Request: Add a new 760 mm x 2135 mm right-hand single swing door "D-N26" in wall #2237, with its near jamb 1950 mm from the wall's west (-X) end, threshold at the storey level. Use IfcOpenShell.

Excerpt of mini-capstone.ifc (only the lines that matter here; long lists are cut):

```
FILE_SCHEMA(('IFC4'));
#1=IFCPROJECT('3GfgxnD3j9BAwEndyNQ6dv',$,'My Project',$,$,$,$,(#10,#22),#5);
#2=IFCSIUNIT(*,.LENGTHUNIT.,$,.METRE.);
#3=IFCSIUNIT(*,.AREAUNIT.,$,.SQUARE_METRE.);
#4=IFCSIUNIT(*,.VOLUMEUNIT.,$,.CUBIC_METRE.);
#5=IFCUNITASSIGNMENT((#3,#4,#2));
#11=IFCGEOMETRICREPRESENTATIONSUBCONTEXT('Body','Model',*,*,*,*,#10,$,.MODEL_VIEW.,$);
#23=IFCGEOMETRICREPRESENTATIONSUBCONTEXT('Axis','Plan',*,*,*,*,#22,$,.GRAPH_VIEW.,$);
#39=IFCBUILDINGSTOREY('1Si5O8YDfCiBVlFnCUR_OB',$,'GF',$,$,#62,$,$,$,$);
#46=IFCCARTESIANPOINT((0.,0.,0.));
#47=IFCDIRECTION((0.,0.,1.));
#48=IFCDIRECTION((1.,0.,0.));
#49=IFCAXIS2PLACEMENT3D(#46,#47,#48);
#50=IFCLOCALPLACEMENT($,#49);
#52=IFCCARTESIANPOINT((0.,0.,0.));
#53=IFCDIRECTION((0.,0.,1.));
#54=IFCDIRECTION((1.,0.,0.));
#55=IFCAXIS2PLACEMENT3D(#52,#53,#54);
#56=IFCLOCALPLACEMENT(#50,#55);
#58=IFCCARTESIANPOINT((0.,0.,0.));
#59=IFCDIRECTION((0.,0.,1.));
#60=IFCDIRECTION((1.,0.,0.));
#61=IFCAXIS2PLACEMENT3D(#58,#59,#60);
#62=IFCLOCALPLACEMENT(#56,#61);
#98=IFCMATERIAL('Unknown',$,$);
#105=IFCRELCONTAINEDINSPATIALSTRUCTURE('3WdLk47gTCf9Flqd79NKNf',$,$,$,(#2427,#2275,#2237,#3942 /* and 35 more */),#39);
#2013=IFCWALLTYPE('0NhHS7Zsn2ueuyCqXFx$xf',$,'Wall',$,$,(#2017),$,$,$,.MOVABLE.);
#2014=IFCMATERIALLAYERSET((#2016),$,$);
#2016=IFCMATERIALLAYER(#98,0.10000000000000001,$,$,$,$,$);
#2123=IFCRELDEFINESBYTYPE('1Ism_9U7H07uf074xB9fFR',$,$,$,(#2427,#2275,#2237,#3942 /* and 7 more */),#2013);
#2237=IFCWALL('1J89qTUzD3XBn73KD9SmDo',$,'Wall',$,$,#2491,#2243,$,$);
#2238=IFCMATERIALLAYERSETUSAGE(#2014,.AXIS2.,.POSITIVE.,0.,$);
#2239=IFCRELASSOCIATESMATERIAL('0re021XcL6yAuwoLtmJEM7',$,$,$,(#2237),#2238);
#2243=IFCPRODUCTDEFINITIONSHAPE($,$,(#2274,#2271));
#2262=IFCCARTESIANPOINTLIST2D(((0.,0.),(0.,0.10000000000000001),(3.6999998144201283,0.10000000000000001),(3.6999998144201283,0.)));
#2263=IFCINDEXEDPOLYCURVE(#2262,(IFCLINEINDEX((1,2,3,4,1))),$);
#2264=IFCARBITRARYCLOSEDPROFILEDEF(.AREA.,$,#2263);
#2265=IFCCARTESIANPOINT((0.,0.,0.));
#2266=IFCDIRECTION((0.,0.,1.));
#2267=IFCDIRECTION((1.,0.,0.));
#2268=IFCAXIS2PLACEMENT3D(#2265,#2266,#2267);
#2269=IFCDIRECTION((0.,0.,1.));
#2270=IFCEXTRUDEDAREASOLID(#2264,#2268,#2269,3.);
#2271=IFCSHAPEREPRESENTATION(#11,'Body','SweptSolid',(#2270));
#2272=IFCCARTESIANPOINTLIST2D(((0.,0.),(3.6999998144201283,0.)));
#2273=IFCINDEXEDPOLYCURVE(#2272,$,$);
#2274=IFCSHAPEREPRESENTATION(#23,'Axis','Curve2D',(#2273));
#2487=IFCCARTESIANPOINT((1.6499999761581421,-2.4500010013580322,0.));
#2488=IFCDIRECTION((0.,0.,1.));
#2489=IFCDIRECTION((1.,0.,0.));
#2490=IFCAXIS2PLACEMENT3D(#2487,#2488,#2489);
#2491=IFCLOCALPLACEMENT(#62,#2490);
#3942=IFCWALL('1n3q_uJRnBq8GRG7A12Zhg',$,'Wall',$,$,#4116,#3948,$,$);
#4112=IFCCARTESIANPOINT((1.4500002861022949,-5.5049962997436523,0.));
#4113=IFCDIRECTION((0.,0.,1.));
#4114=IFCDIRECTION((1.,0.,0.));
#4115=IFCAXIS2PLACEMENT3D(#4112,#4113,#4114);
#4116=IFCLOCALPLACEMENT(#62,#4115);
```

```python
import numpy as np
import ifcopenshell
import ifcopenshell.api.feature
import ifcopenshell.api.geometry
import ifcopenshell.api.root
import ifcopenshell.api.spatial
import ifcopenshell.geom
import ifcopenshell.util.element
import ifcopenshell.util.placement
import ifcopenshell.util.representation
import ifcopenshell.util.shape
import ifcopenshell.util.unit

model = ifcopenshell.open("mini-capstone.ifc")
unit_scale = ifcopenshell.util.unit.calculate_unit_scale(model)
settings = ifcopenshell.geom.settings()


def volume(element):
    """Net volume in cubic metres, openings subtracted."""
    shape = ifcopenshell.geom.create_shape(settings, element)
    return ifcopenshell.util.shape.get_volume(shape.geometry)


wall = model.by_guid("1J89qTUzD3XBn73KD9SmDo")
storey = ifcopenshell.util.element.get_container(wall, ifc_class="IfcBuildingStorey")
context = ifcopenshell.util.representation.get_context(model, "Model", "Body", "MODEL_VIEW")
before = volume(wall)

width, height, from_end, sill = 0.76, 2.135, 1.95, 0.0  # metres

# The wall runs along its own X axis, and the end named is its -X end.
wall_shape = ifcopenshell.geom.create_shape(settings, wall)
x, y, z = ifcopenshell.util.shape.get_vertices(wall_shape.geometry).T
start = x.min() + from_end
face, thickness = float(y.min()), float(y.max() - y.min())
wall_matrix = ifcopenshell.util.placement.get_local_placement(wall.ObjectPlacement)
level = ifcopenshell.util.placement.get_local_placement(storey.ObjectPlacement)[2, 3]


def in_wall(x, y):
    """Placement at x, y metres in the wall's axes, at sill height."""
    matrix = wall_matrix.copy()
    matrix[:, 3] = wall_matrix @ np.array([x / unit_scale, y / unit_scale, 0.0, 1.0])
    matrix[2, 3] = level + sill / unit_scale
    return matrix


# Opening: a box that overshoots both wall faces by 50 mm.
opening = ifcopenshell.api.root.create_entity(model, ifc_class="IfcOpeningElement", predefined_type="OPENING")
box = ifcopenshell.api.geometry.add_wall_representation(
    model, context=context, length=width, height=height, thickness=thickness + 0.1
)
ifcopenshell.api.geometry.assign_representation(model, product=opening, representation=box)
ifcopenshell.api.geometry.edit_object_placement(model, product=opening, matrix=in_wall(start, face - 0.05), is_si=False)
ifcopenshell.api.feature.add_feature(model, feature=opening, element=wall)

door = ifcopenshell.api.root.create_entity(model, ifc_class="IfcDoor", name="D-N26", predefined_type="DOOR")
door.OverallWidth, door.OverallHeight = width / unit_scale, height / unit_scale
door.OperationType = "SINGLE_SWING_RIGHT"
body = ifcopenshell.api.geometry.add_door_representation(
    model,
    context=context,
    overall_width=door.OverallWidth,
    overall_height=door.OverallHeight,
    operation_type="SINGLE_SWING_RIGHT",
    lining_properties={"LiningDepth": thickness / unit_scale, "ThresholdDepth": thickness / unit_scale},
)
ifcopenshell.api.geometry.assign_representation(model, product=door, representation=body)
ifcopenshell.api.spatial.assign_container(model, products=[door], relating_structure=storey)
ifcopenshell.api.feature.add_filling(model, opening=opening, element=door)

# The lining spans the wall, so the door starts at the wall face.
ifcopenshell.api.geometry.edit_object_placement(model, product=door, matrix=in_wall(start, face), is_si=False)

after = volume(wall)

print(f"wall volume {before:.3f} -> {after:.3f} m3")

model.write("mini-capstone-out.ifc")
```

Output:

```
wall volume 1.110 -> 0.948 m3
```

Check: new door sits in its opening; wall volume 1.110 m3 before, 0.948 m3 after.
